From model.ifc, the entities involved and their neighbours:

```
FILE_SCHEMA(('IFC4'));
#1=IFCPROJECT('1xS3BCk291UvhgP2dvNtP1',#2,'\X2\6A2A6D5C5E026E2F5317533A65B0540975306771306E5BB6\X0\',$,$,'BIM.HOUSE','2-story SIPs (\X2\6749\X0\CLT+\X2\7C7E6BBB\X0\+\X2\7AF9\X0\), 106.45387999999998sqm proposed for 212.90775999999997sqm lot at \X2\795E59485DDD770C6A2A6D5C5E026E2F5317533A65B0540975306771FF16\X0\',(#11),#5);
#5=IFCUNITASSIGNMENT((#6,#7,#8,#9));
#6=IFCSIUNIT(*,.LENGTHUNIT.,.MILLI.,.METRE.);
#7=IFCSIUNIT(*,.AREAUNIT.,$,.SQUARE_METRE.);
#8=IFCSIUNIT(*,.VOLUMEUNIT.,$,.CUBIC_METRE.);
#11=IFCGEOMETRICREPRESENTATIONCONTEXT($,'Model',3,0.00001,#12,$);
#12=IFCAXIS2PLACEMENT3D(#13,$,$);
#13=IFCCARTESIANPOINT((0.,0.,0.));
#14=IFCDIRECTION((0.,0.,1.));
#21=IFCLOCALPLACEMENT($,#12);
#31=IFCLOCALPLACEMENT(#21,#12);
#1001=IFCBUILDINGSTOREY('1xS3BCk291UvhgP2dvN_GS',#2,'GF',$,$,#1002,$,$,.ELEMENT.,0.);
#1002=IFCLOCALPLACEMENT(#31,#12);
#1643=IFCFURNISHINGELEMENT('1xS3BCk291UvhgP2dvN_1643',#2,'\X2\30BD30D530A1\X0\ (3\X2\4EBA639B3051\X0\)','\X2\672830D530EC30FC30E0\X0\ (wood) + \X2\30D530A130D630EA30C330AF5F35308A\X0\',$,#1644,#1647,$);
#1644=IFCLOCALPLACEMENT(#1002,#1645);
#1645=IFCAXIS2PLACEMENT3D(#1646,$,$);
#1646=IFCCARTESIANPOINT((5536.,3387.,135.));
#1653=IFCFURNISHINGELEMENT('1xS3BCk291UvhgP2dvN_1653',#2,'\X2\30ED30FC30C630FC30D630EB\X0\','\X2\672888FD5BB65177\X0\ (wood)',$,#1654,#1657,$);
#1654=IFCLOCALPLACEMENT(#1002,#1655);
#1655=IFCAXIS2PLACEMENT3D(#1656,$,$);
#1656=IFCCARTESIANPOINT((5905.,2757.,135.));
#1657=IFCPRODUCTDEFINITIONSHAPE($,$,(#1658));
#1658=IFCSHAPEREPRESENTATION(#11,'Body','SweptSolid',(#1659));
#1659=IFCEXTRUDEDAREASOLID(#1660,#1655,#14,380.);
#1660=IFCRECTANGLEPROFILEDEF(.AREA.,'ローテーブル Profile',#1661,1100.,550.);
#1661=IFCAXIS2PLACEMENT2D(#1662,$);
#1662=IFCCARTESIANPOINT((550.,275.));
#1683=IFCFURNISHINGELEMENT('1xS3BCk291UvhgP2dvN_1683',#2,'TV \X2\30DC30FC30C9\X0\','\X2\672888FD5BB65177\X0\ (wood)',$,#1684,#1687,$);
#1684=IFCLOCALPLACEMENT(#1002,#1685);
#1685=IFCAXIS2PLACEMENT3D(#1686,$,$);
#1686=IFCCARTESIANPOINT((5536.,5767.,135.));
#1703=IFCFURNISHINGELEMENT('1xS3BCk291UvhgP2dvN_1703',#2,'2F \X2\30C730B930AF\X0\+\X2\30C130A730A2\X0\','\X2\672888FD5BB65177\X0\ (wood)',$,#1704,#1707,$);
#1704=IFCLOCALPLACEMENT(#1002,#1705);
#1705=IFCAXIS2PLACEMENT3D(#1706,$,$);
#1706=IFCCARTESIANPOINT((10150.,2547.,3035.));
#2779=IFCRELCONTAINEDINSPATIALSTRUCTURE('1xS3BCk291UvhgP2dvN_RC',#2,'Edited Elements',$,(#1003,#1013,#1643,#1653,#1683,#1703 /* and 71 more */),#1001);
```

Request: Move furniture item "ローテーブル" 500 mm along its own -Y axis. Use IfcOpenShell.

```python
import ifcopenshell
import ifcopenshell.api.geometry
import ifcopenshell.util.placement
import ifcopenshell.util.unit

model = ifcopenshell.open("model.ifc")
unit_scale = ifcopenshell.util.unit.calculate_unit_scale(model)

item = model.by_id(1653)
matrix = ifcopenshell.util.placement.get_local_placement(item.ObjectPlacement)
matrix[:3, 3] -= matrix[:3, 1] * 0.5 / unit_scale
ifcopenshell.api.geometry.edit_object_placement(model, product=item, matrix=matrix, is_si=False)

print(ifcopenshell.util.placement.get_local_placement(item.ObjectPlacement).round(3) + 0.0)

model.write("model-out.ifc")
```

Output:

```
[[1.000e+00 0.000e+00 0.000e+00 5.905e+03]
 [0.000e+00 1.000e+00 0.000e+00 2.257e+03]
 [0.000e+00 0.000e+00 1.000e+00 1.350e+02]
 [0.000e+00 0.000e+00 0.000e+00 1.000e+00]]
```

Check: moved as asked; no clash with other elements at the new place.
